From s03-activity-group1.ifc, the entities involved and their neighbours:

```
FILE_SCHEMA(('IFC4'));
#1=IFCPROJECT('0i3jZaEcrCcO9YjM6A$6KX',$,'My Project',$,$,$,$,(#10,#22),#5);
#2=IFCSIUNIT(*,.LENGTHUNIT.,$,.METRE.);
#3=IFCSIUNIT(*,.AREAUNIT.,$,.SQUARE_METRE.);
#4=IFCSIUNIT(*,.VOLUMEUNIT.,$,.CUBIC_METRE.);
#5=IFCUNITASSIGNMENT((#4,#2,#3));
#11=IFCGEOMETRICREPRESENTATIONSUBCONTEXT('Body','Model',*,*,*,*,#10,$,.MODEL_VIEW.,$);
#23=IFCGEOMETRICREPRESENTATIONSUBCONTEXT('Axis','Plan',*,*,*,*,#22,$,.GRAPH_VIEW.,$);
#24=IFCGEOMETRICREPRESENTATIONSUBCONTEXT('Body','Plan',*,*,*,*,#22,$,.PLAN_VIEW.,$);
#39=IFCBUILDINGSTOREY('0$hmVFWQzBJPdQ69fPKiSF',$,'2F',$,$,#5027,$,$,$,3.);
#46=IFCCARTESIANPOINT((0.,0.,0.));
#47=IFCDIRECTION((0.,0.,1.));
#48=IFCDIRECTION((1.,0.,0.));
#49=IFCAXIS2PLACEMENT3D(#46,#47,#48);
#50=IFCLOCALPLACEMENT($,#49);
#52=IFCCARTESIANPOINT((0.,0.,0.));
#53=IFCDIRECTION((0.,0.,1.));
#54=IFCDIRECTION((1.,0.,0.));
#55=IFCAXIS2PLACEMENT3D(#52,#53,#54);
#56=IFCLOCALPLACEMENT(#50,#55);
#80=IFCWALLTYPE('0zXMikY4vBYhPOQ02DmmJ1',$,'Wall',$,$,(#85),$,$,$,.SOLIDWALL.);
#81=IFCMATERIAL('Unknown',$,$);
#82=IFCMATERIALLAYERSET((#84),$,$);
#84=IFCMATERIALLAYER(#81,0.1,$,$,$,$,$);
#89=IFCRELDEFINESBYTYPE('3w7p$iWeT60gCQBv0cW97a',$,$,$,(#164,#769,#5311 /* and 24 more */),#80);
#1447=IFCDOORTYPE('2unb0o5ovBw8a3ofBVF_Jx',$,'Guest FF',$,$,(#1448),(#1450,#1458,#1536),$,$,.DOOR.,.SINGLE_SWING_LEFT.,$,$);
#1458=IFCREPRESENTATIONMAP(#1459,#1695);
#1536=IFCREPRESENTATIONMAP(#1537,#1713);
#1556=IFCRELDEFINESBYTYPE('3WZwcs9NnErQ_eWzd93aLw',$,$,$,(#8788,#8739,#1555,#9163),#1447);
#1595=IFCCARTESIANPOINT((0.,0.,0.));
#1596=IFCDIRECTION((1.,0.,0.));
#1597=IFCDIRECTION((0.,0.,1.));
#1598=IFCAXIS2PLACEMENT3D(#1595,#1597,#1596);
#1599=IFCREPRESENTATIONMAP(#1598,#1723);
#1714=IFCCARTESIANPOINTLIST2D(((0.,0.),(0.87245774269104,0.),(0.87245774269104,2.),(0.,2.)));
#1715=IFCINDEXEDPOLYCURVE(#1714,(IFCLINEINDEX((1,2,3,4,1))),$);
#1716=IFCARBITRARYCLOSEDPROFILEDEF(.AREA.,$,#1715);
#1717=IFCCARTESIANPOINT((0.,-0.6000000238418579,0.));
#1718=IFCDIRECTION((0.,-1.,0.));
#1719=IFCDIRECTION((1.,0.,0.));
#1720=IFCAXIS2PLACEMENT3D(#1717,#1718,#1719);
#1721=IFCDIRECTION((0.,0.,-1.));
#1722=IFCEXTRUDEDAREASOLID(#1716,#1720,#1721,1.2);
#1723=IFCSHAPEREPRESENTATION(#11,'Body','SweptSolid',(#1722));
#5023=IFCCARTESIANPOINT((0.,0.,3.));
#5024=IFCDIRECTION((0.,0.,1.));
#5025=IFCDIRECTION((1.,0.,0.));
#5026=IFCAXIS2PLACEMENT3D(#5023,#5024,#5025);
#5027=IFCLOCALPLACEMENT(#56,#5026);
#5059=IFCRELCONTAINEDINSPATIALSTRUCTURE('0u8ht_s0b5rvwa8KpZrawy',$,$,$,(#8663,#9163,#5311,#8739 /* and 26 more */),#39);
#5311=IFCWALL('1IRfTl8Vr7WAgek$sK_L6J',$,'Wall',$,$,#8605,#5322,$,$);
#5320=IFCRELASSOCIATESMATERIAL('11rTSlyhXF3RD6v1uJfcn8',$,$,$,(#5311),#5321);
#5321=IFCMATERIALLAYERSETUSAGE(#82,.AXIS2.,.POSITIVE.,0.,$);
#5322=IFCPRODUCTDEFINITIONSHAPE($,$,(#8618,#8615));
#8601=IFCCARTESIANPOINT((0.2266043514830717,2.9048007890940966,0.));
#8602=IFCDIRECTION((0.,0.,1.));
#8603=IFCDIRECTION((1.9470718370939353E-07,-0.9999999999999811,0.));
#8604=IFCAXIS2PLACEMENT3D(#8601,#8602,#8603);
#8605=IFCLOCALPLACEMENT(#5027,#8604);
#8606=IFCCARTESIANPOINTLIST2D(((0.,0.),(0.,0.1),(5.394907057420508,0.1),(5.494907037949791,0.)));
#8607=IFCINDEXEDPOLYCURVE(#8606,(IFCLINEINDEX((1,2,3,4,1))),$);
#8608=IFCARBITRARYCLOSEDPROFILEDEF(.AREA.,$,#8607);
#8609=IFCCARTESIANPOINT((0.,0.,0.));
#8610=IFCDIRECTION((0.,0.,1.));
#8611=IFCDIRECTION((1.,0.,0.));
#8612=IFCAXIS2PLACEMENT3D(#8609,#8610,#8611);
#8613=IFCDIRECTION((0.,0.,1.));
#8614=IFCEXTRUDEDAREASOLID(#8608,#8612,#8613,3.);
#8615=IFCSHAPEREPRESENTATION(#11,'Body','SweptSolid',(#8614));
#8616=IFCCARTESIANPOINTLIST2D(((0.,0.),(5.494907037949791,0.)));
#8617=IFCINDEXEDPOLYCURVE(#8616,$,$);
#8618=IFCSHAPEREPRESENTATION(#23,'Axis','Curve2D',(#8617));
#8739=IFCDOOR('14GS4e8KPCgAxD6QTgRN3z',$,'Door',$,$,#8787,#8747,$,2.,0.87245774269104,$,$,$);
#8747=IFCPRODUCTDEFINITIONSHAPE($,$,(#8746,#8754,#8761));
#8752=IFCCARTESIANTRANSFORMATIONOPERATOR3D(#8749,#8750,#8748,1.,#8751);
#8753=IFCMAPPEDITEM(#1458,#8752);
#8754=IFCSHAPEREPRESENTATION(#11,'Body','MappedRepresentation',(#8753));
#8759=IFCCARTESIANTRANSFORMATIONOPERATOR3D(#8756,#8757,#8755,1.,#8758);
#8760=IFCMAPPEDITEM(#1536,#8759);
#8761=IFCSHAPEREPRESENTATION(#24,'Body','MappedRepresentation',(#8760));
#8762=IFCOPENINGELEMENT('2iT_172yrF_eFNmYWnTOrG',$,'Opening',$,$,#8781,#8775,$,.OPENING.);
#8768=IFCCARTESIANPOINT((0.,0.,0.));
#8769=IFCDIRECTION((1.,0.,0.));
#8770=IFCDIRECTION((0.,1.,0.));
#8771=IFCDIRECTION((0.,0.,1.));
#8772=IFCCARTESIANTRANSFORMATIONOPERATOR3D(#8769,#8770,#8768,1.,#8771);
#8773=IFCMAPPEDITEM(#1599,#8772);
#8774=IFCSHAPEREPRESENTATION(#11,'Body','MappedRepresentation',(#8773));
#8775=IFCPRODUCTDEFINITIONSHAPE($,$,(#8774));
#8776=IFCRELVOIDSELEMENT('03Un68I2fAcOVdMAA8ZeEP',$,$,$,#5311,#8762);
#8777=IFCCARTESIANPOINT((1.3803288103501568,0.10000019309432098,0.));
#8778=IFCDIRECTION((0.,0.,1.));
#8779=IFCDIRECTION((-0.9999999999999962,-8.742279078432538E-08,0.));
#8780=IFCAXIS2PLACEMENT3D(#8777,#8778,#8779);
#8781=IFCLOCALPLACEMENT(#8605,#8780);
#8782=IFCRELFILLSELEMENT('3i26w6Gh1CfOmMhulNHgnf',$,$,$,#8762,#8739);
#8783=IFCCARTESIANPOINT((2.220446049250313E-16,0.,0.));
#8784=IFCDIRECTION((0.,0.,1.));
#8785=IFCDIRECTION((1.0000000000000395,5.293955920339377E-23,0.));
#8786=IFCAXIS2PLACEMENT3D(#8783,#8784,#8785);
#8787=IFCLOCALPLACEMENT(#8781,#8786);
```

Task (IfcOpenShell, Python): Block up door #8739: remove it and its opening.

```python
import ifcopenshell
import ifcopenshell.api.feature
import ifcopenshell.api.root
import ifcopenshell.geom
import ifcopenshell.util.shape

model = ifcopenshell.open("s03-activity-group1.ifc")
settings = ifcopenshell.geom.settings()


def volume(element):
    """Net volume in cubic metres, openings subtracted."""
    shape = ifcopenshell.geom.create_shape(settings, element)
    return ifcopenshell.util.shape.get_volume(shape.geometry)


door = model.by_id(8739)
opening = door.FillsVoids[0].RelatingOpeningElement
wall = opening.VoidsElements[0].RelatingBuildingElement
before = volume(wall)

ifcopenshell.api.root.remove_product(model, product=door)
ifcopenshell.api.feature.remove_feature(model, feature=opening)

after = volume(wall)

print(f"wall volume {before:.3f} -> {after:.3f} m3")

model.write("s03-activity-group1_edited.ifc")
```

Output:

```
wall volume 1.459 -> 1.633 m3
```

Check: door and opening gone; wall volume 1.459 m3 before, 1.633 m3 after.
